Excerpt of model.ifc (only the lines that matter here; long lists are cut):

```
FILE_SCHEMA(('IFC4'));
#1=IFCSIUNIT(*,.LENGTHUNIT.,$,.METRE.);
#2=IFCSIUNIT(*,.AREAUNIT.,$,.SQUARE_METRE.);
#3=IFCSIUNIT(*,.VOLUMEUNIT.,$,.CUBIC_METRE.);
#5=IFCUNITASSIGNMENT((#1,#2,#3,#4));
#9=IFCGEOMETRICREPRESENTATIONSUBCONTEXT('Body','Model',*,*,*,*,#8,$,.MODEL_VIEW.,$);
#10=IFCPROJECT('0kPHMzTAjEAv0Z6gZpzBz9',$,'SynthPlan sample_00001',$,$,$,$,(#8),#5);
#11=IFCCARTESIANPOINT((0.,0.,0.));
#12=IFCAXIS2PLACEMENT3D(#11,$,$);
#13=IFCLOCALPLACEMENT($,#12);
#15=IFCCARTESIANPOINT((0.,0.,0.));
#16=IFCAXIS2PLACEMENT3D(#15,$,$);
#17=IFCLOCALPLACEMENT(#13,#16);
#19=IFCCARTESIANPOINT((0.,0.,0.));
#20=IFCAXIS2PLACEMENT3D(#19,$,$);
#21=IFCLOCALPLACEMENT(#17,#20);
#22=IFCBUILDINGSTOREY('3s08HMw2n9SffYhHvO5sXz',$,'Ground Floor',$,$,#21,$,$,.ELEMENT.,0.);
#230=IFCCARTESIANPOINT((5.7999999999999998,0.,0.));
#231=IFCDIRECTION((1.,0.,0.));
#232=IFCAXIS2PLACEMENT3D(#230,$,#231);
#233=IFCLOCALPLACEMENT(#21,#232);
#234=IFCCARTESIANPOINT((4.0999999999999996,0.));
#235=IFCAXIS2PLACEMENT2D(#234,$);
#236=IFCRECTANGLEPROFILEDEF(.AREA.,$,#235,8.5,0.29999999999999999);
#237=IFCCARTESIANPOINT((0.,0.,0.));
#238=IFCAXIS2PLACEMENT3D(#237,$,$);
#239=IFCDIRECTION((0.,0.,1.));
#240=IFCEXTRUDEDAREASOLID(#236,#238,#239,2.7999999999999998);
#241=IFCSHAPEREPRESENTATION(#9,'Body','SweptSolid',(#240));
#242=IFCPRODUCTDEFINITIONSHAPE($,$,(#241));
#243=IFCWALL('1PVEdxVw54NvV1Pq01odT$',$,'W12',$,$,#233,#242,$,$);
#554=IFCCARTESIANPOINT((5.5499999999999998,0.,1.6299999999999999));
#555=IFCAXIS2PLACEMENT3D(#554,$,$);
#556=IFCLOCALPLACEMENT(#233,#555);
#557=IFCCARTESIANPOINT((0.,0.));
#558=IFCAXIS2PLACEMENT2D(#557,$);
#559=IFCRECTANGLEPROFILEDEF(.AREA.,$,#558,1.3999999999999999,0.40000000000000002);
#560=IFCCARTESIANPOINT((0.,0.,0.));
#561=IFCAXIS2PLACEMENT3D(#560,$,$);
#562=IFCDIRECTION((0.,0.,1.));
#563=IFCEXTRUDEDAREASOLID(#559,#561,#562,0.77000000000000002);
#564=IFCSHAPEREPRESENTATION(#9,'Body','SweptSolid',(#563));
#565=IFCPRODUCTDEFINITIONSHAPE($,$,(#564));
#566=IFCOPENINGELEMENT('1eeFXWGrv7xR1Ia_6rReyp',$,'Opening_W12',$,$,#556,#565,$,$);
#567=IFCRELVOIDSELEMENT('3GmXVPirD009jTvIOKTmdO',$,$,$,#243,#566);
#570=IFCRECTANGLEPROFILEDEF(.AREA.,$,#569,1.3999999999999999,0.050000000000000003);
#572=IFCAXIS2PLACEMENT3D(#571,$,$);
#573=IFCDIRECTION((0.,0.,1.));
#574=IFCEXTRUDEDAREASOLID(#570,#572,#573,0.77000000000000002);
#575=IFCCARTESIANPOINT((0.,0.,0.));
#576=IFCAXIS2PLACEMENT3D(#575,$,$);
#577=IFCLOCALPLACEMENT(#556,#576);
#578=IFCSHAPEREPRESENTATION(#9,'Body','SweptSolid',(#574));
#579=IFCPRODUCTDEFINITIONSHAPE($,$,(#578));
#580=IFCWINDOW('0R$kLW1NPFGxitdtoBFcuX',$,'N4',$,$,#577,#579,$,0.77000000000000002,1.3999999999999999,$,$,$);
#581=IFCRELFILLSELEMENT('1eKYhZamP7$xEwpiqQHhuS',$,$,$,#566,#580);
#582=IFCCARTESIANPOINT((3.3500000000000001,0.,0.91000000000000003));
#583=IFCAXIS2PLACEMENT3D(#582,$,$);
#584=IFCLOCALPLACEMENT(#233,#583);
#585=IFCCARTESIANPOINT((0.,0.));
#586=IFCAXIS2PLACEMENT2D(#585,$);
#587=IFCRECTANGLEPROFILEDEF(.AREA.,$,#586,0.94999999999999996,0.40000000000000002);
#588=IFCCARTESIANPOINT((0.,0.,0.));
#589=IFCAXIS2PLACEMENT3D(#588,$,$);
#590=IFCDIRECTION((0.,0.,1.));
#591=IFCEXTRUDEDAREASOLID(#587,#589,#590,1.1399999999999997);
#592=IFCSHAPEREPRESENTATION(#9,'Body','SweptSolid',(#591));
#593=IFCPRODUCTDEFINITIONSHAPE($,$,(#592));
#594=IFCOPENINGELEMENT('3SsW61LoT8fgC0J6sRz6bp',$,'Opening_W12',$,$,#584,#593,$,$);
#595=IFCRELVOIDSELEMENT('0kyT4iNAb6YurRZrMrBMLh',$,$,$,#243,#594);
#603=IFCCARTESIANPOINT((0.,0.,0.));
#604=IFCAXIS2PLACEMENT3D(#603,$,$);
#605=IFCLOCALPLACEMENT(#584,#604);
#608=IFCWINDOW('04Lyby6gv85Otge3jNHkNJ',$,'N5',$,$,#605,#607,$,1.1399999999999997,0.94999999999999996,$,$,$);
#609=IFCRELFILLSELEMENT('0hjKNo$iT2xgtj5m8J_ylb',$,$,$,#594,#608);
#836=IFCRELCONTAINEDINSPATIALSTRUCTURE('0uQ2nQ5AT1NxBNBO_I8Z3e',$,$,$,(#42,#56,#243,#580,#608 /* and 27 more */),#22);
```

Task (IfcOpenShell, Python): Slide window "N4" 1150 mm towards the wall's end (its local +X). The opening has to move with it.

```python
import ifcopenshell
import ifcopenshell.api.geometry
import ifcopenshell.util.placement

model = ifcopenshell.open("model.ifc")

window = model.by_guid("0R$kLW1NPFGxitdtoBFcuX")
opening = window.FillsVoids[0].RelatingOpeningElement
wall = opening.VoidsElements[0].RelatingBuildingElement

wall_matrix = ifcopenshell.util.placement.get_local_placement(wall.ObjectPlacement)
shift = wall_matrix[:3, 0] * 1.15
before = ifcopenshell.util.placement.get_local_placement(window.ObjectPlacement)[:3, 3].copy()

# The window is placed relative to its opening, so it follows when the opening moves.
matrix = ifcopenshell.util.placement.get_local_placement(opening.ObjectPlacement)
matrix[:3, 3] += shift
ifcopenshell.api.geometry.edit_object_placement(
    model, product=opening, matrix=matrix, is_si=False, should_transform_children=True
)

after = ifcopenshell.util.placement.get_local_placement(window.ObjectPlacement)[:3, 3]
print("window moved by", (after - before).round(3) + 0.0)

model.write("model_v2.ifc")
```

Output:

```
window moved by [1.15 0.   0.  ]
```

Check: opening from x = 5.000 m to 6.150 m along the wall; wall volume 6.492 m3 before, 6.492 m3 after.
